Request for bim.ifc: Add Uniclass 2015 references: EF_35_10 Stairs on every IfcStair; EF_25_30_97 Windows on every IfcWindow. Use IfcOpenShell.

First a look at what the model holds.

```python
import ifcopenshell

model = ifcopenshell.open("bim.ifc")
print(model.schema)
print("classifications:", [c.Name for c in model.by_type("IfcClassification")])
for ifc_class in ("IfcDoor", "IfcRoof", "IfcStair", "IfcWall", "IfcWindow"):
    print(ifc_class, len(model.by_type(ifc_class)))
```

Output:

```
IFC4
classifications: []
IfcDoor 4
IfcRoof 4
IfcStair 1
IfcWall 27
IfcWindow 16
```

```python
import ifcopenshell
import ifcopenshell.api.classification

model = ifcopenshell.open("bim.ifc")

system = ifcopenshell.api.classification.add_classification(model, classification="Uniclass 2015")

codes = {
    "IfcStair": ("EF_35_10", "Stairs"),
    "IfcWindow": ("EF_25_30_97", "Windows"),
}
for ifc_class, (code, name) in codes.items():
    products = model.by_type(ifc_class)
    ifcopenshell.api.classification.add_reference(
        model, products=products, classification=system, identification=code, name=name
    )
    print(code, len(products))

model.write("bim_v2.ifc")
```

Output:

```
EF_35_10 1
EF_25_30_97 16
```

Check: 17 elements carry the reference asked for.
